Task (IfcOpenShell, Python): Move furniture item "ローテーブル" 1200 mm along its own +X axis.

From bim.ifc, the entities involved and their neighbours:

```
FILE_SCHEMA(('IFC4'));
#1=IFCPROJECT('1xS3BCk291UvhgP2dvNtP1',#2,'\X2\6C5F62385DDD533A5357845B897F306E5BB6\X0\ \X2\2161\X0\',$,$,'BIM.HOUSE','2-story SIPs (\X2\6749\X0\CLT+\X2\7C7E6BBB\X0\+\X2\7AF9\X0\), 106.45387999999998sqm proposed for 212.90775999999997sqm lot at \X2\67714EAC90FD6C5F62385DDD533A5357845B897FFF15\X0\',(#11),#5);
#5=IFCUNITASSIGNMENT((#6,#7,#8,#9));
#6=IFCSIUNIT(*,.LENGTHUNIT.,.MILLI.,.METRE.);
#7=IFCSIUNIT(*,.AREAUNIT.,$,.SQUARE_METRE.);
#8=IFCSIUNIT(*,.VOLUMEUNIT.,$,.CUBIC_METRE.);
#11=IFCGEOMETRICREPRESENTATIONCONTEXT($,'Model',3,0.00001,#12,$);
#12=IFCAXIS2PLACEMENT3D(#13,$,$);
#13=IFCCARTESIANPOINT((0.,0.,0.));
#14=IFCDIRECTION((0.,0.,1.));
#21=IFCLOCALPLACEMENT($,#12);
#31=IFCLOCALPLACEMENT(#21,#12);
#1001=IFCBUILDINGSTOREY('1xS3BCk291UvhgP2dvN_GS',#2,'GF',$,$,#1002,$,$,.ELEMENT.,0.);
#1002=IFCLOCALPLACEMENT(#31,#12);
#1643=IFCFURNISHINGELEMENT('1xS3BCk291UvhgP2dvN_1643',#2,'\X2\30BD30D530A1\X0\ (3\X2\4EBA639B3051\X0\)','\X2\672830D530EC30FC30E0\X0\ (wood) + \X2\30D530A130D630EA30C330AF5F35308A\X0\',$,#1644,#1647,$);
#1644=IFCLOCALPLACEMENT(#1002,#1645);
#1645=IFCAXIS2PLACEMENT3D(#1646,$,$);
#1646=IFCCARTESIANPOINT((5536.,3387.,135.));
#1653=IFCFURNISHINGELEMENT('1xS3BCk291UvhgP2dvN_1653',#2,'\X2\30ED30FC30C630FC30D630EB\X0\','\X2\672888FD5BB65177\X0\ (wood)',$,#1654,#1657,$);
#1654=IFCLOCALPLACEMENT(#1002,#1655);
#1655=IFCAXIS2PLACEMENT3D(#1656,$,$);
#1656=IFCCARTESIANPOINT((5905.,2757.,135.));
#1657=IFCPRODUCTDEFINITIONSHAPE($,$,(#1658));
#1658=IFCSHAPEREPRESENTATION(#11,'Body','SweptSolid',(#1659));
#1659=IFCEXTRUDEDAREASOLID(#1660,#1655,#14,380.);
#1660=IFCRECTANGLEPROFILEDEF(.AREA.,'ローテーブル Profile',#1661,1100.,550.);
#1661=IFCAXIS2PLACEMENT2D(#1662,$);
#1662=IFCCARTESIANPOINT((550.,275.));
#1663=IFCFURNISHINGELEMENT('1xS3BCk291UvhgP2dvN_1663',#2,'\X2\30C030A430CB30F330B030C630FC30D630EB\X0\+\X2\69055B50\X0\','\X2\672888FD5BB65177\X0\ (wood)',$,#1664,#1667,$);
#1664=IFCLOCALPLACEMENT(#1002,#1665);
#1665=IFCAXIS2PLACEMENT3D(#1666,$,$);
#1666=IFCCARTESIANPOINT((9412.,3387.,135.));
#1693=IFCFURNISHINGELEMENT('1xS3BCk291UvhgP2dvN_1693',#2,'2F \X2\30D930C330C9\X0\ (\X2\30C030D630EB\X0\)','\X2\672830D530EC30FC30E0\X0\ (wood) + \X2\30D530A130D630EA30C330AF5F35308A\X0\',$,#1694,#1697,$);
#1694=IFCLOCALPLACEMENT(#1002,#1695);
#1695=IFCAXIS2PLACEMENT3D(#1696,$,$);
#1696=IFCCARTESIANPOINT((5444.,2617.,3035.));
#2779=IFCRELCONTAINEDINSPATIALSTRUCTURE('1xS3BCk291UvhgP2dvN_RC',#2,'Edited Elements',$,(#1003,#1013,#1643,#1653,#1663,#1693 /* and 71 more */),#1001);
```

```python
import ifcopenshell
import ifcopenshell.api.geometry
import ifcopenshell.util.placement

model = ifcopenshell.open("bim.ifc")

item = model.by_id(1653)
matrix = ifcopenshell.util.placement.get_local_placement(item.ObjectPlacement)
matrix[:3, 3] += matrix[:3, 0] * 1200.0
ifcopenshell.api.geometry.edit_object_placement(model, product=item, matrix=matrix, is_si=False)

print(ifcopenshell.util.placement.get_local_placement(item.ObjectPlacement).round(3) + 0.0)

model.write("bim_v2.ifc")
```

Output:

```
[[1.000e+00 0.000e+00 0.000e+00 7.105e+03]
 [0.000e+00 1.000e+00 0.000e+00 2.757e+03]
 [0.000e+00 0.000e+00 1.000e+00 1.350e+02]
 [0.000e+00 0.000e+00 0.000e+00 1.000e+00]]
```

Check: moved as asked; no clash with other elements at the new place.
